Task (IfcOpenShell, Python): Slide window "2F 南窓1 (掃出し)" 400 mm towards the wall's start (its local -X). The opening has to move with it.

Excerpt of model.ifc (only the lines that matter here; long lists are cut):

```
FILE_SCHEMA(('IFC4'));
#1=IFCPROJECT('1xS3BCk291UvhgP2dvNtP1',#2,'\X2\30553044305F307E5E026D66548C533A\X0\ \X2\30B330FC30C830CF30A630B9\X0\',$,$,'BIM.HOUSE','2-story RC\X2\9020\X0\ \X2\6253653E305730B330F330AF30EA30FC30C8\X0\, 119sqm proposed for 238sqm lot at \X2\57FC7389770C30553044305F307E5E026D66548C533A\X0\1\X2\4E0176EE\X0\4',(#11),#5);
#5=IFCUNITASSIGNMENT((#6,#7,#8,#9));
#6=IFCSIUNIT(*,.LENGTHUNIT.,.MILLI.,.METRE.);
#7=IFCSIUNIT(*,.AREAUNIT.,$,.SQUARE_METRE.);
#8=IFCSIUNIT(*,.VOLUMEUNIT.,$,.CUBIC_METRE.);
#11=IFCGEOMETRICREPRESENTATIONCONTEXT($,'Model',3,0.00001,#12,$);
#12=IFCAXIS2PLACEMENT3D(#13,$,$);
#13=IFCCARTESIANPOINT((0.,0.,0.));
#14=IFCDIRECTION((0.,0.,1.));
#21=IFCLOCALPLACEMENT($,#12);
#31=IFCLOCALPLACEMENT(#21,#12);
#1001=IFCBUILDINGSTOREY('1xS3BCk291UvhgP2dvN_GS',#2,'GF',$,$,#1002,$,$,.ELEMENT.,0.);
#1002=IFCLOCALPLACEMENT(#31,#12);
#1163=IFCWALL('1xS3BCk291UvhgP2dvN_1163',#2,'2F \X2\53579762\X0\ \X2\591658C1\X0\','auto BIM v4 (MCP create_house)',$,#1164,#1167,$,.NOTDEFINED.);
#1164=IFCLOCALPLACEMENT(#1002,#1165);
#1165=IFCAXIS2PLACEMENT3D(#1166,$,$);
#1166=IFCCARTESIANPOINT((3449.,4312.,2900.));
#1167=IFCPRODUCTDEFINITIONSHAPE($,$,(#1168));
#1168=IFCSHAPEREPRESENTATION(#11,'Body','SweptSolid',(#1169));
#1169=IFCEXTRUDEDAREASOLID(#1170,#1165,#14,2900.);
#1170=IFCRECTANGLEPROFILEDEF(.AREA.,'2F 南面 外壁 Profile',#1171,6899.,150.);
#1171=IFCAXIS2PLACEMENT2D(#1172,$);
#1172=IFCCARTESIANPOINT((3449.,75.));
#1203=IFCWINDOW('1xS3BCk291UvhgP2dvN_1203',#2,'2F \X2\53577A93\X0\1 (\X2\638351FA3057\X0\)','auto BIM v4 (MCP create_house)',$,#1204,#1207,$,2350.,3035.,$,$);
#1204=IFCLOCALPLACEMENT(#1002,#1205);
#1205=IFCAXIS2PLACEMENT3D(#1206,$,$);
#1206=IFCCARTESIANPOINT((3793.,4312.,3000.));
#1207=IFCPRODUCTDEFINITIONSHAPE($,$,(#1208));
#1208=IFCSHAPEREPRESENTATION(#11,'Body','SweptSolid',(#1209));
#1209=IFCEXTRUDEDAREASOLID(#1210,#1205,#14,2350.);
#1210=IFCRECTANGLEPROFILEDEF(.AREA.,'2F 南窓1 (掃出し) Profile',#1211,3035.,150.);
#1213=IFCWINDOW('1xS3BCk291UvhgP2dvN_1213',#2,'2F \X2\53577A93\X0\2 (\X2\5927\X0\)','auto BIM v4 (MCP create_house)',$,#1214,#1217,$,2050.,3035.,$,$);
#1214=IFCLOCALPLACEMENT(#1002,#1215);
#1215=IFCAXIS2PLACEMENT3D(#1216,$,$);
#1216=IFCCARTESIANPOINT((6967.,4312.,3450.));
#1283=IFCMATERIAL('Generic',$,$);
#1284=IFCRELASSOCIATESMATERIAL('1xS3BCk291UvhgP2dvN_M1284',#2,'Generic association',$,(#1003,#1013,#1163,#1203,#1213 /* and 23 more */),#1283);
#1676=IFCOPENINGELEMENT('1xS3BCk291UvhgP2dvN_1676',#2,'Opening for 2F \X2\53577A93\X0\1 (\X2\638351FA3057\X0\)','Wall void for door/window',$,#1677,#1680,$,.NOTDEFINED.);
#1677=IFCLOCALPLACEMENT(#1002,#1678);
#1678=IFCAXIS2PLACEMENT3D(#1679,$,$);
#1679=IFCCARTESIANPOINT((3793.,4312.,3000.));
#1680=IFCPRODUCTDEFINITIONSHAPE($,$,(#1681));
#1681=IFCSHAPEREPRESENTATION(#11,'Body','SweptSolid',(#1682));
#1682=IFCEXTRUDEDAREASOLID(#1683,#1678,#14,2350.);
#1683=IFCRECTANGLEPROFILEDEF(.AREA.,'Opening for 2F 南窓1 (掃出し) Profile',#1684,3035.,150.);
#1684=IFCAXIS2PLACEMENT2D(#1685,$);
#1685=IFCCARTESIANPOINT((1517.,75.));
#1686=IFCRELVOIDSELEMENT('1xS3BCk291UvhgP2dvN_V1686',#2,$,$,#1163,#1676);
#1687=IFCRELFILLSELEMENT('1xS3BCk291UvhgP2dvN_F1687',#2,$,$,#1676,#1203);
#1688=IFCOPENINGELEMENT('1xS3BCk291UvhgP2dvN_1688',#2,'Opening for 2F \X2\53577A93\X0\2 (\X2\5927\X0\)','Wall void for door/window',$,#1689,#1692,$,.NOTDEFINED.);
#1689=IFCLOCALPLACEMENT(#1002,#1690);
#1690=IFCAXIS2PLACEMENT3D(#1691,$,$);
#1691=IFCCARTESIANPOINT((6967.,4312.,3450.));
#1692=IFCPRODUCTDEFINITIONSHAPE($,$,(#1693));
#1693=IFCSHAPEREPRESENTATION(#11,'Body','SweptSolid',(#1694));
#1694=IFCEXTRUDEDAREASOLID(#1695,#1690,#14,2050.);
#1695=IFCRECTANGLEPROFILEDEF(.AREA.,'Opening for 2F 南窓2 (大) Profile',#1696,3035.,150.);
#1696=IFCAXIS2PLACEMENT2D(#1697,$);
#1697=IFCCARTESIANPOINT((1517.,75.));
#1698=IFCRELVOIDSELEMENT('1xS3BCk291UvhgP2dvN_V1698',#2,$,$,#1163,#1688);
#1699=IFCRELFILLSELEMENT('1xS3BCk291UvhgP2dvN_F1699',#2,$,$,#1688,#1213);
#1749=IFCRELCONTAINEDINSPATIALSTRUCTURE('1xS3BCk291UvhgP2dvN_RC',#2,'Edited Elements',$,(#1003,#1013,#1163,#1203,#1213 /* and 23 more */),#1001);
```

```python
import ifcopenshell
import ifcopenshell.api.geometry
import ifcopenshell.util.placement

model = ifcopenshell.open("model.ifc")

window = model.by_guid("1xS3BCk291UvhgP2dvN_1203")
opening = window.FillsVoids[0].RelatingOpeningElement
wall = opening.VoidsElements[0].RelatingBuildingElement

wall_matrix = ifcopenshell.util.placement.get_local_placement(wall.ObjectPlacement)
shift = wall_matrix[:3, 0] * -400.0
before = ifcopenshell.util.placement.get_local_placement(window.ObjectPlacement)[:3, 3].copy()

# The window is not placed relative to its opening, so move both.
for product in (opening, window):
    matrix = ifcopenshell.util.placement.get_local_placement(product.ObjectPlacement)
    matrix[:3, 3] += shift
    ifcopenshell.api.geometry.edit_object_placement(model, product=product, matrix=matrix, is_si=False)

after = ifcopenshell.util.placement.get_local_placement(window.ObjectPlacement)[:3, 3]
print("window moved by", (after - before).round(3) + 0.0)

model.write("model_updated.ifc")
```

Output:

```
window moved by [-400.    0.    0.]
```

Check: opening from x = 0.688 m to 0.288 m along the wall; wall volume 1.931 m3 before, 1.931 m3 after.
